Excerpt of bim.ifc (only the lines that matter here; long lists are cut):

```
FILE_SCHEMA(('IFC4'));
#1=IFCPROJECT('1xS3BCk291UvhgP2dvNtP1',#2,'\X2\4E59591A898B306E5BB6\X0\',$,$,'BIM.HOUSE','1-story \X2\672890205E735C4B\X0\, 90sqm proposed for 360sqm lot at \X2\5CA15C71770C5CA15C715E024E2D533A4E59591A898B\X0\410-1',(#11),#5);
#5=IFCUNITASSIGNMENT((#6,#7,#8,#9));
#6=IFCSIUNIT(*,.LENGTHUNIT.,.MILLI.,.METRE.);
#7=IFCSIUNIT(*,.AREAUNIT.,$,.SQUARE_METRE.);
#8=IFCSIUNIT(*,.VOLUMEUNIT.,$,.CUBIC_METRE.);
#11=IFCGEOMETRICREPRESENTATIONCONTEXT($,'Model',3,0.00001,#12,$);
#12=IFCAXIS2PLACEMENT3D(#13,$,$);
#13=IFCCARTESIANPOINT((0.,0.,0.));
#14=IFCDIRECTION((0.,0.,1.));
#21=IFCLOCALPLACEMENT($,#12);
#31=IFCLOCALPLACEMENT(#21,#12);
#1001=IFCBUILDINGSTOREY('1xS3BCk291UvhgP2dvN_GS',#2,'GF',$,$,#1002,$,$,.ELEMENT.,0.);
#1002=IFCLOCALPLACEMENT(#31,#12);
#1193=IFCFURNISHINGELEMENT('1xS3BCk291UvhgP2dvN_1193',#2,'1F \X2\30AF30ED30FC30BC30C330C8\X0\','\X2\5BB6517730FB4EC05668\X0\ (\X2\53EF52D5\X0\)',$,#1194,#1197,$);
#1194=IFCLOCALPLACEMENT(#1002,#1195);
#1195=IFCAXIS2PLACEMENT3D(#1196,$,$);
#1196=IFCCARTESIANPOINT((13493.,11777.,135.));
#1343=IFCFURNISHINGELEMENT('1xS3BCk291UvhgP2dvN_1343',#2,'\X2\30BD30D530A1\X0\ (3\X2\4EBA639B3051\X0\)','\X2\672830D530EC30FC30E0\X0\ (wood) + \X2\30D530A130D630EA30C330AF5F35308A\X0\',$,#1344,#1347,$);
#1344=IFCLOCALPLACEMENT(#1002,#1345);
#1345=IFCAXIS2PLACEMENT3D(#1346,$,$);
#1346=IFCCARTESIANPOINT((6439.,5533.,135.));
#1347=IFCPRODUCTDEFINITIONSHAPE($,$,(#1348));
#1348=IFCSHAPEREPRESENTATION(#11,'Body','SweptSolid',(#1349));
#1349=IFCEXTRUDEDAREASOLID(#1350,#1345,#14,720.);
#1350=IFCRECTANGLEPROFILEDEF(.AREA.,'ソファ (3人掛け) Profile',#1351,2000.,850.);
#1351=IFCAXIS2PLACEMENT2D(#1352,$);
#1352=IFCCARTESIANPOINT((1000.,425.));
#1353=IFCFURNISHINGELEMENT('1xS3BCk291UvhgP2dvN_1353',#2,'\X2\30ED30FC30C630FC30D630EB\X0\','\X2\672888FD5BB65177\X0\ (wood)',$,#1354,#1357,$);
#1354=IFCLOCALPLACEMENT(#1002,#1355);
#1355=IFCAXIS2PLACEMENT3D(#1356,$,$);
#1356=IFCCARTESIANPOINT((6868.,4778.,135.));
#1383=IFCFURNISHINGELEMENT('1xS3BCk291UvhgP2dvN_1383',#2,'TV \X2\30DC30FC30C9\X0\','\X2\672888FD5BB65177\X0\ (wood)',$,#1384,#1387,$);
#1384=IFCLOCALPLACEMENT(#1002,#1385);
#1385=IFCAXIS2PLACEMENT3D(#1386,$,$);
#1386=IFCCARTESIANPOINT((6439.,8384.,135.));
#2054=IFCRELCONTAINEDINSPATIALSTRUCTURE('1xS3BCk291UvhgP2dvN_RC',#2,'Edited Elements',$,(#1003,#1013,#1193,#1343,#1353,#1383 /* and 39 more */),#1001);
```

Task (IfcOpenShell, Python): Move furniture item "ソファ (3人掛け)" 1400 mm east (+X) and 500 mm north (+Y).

```python
import ifcopenshell
import ifcopenshell.api.geometry
import ifcopenshell.util.placement
import ifcopenshell.util.unit

model = ifcopenshell.open("bim.ifc")
unit_scale = ifcopenshell.util.unit.calculate_unit_scale(model)

item = model.by_id(1343)
matrix = ifcopenshell.util.placement.get_local_placement(item.ObjectPlacement)
matrix[0, 3] += 1.4 / unit_scale
matrix[1, 3] += 0.5 / unit_scale
ifcopenshell.api.geometry.edit_object_placement(model, product=item, matrix=matrix, is_si=False)

print(ifcopenshell.util.placement.get_local_placement(item.ObjectPlacement).round(3) + 0.0)

model.write("bim-out.ifc")
```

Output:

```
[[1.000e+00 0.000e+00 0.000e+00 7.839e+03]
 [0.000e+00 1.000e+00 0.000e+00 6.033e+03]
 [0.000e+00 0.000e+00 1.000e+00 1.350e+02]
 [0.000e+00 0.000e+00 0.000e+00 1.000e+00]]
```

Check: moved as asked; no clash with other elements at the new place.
